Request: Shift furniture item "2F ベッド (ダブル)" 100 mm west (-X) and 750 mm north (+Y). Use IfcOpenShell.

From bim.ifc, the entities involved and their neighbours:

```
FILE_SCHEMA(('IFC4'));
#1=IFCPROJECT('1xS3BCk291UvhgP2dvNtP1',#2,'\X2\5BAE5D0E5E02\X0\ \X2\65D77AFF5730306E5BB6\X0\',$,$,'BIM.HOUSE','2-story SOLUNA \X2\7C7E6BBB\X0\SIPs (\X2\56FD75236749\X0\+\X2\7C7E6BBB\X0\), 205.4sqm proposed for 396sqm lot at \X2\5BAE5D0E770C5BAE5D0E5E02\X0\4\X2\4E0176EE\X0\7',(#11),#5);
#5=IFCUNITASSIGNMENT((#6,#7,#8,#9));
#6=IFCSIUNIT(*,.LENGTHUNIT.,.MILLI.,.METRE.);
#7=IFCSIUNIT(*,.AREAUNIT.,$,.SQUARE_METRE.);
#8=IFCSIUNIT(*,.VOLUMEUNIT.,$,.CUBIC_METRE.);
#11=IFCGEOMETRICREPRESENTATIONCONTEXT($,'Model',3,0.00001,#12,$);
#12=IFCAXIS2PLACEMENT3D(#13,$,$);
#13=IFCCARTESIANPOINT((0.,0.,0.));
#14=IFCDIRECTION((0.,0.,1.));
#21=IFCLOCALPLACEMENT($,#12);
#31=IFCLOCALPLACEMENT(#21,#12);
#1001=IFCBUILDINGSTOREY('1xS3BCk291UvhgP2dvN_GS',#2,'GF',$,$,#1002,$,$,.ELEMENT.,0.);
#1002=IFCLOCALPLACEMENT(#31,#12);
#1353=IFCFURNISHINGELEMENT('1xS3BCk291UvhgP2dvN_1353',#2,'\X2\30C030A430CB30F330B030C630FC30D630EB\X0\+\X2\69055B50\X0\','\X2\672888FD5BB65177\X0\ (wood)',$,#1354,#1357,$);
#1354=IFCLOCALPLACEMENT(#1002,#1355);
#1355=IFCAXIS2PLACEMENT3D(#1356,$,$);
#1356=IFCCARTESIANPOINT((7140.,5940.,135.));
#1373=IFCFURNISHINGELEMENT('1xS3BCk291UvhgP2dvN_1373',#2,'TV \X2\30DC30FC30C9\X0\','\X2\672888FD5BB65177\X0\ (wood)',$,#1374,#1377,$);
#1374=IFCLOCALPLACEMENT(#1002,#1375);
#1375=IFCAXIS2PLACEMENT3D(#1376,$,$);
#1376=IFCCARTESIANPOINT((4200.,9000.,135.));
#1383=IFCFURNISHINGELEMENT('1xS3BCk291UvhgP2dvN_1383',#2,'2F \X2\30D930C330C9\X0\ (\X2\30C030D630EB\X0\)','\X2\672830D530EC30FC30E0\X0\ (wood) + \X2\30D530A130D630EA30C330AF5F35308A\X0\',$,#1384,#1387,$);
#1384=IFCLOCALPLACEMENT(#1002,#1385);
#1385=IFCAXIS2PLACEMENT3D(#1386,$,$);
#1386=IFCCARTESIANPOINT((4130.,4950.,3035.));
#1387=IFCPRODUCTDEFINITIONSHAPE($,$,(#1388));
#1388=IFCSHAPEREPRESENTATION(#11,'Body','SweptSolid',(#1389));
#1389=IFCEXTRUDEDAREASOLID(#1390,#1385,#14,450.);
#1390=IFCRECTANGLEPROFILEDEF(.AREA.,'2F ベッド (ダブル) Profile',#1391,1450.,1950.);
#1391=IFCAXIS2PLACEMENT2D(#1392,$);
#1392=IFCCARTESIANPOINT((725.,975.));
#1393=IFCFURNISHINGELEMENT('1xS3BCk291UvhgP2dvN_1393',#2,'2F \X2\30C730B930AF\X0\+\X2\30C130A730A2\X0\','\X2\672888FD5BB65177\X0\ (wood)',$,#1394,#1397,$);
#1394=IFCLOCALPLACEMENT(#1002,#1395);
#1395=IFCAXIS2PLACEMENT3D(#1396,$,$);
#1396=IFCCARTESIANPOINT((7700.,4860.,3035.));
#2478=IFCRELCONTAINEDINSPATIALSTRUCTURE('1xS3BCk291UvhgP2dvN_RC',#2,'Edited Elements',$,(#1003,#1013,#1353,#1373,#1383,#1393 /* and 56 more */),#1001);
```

```python
import ifcopenshell
import ifcopenshell.api.geometry
import ifcopenshell.util.placement

model = ifcopenshell.open("bim.ifc")

item = model.by_id(1383)
matrix = ifcopenshell.util.placement.get_local_placement(item.ObjectPlacement)
matrix[0, 3] -= 100.0
matrix[1, 3] += 750.0
ifcopenshell.api.geometry.edit_object_placement(model, product=item, matrix=matrix, is_si=False)

print(ifcopenshell.util.placement.get_local_placement(item.ObjectPlacement).round(3) + 0.0)

model.write("bim-out.ifc")
```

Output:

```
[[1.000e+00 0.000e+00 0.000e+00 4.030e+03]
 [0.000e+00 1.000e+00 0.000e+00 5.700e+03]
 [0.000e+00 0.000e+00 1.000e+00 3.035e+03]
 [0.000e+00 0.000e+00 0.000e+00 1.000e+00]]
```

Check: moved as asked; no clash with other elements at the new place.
